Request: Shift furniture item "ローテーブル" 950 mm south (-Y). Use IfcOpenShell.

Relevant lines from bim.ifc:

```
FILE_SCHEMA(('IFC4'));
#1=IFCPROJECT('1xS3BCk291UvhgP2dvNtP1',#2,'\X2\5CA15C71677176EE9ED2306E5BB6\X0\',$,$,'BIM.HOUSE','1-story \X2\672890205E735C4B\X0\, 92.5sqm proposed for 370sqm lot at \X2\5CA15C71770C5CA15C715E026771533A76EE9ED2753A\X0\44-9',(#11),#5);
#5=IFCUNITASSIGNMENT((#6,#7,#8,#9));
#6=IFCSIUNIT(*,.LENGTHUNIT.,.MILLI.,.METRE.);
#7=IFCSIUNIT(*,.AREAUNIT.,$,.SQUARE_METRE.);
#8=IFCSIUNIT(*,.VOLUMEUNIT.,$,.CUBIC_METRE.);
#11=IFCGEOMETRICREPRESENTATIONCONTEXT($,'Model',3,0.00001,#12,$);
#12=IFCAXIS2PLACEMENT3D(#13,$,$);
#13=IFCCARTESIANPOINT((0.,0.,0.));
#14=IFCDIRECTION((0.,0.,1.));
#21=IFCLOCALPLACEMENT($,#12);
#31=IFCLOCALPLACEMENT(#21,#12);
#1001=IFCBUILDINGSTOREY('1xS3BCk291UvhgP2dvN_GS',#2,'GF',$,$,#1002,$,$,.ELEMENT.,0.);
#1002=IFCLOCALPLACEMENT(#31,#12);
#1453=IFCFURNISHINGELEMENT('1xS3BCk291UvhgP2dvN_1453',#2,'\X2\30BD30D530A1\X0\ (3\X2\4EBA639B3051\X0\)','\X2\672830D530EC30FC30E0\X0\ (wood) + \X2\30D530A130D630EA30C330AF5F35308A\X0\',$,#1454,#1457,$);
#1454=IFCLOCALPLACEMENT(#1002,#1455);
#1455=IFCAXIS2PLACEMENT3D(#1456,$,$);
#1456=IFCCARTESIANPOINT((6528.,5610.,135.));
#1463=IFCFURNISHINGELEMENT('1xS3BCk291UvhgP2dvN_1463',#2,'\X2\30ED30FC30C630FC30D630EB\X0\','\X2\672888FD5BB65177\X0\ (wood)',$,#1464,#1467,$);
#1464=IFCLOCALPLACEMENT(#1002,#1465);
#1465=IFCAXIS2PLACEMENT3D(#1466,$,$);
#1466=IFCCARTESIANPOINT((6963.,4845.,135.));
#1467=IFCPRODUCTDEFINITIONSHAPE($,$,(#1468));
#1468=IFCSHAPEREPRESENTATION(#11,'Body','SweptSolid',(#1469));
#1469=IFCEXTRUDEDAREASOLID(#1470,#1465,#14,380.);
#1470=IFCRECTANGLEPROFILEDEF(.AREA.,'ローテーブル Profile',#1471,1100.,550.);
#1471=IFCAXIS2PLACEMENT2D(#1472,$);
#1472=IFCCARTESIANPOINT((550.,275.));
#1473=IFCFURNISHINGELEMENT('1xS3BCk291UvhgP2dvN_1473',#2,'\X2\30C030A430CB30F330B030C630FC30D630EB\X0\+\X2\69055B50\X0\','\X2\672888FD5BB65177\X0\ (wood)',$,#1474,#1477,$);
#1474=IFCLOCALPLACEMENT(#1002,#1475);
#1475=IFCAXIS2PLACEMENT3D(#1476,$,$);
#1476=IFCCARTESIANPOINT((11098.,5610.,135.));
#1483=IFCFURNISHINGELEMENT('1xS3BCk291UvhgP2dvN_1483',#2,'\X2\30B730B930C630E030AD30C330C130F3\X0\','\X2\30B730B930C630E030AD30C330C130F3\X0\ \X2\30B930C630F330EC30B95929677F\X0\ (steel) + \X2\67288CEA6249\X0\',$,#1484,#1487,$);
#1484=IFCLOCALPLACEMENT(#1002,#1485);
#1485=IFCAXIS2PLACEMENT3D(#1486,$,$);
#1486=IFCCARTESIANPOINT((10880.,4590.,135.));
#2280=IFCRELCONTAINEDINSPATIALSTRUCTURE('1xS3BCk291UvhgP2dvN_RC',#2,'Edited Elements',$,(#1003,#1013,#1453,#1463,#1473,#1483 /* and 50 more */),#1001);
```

```python
import ifcopenshell
import ifcopenshell.api.geometry
import ifcopenshell.util.placement
import ifcopenshell.util.unit

model = ifcopenshell.open("bim.ifc")
unit_scale = ifcopenshell.util.unit.calculate_unit_scale(model)

item = model.by_id(1463)
matrix = ifcopenshell.util.placement.get_local_placement(item.ObjectPlacement)
matrix[1, 3] -= 0.95 / unit_scale
ifcopenshell.api.geometry.edit_object_placement(model, product=item, matrix=matrix, is_si=False)

print(ifcopenshell.util.placement.get_local_placement(item.ObjectPlacement).round(3) + 0.0)

model.write("bim_v2.ifc")
```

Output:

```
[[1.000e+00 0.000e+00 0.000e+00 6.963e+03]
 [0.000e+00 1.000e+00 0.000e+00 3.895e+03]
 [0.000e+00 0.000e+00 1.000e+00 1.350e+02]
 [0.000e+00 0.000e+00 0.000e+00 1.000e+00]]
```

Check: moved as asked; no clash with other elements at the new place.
